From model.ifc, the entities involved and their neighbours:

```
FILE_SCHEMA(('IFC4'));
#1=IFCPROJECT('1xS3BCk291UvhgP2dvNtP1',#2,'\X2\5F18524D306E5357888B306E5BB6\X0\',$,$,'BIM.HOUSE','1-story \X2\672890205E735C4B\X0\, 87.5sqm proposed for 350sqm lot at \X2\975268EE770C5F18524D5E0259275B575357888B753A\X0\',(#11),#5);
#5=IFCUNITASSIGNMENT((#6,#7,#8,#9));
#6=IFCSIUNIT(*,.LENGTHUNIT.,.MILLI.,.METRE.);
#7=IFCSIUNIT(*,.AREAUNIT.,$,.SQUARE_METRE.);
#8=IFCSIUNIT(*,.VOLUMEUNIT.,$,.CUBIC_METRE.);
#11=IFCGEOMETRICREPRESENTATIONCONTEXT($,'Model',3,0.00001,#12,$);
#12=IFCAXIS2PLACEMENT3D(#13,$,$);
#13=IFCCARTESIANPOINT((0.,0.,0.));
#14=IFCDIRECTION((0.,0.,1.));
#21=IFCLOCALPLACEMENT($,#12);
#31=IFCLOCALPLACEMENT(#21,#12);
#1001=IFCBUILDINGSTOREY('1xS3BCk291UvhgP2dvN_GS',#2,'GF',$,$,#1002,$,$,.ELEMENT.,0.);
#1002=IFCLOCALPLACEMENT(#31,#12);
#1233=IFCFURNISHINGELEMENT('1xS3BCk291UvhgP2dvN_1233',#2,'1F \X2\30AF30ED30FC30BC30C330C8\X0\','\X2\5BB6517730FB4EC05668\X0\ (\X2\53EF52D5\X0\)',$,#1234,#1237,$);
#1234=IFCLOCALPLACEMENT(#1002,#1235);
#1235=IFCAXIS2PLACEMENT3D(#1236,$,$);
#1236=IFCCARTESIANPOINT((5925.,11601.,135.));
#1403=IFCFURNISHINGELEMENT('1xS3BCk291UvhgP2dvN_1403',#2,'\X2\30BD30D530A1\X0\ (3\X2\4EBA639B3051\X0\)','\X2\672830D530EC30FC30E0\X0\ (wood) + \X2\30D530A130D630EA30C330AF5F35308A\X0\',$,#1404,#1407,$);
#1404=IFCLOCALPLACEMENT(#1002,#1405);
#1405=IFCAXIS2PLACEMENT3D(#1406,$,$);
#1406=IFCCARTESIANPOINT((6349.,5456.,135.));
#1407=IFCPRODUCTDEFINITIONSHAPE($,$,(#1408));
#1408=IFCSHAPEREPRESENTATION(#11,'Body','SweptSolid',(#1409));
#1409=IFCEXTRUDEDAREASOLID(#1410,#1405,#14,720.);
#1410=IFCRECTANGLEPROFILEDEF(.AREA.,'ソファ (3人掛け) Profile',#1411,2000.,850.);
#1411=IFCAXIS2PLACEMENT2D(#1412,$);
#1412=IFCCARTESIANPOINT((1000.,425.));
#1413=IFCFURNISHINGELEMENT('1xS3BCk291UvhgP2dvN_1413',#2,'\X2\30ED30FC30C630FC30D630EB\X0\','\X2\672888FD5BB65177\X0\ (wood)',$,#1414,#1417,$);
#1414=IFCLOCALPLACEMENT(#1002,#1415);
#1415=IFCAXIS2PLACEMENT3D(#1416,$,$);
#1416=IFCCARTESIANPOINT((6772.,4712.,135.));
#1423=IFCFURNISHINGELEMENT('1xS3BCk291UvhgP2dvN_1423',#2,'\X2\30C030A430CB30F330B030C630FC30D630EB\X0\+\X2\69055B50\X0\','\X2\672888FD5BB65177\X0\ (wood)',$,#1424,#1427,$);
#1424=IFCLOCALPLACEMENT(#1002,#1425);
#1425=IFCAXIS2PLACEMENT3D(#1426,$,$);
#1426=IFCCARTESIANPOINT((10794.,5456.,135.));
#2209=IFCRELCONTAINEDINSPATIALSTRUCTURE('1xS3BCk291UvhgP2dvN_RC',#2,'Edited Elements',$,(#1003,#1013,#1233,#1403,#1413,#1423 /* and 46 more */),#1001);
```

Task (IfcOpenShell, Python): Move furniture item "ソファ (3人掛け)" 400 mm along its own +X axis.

```python
import ifcopenshell
import ifcopenshell.api.geometry
import ifcopenshell.util.placement
import ifcopenshell.util.unit

model = ifcopenshell.open("model.ifc")
unit_scale = ifcopenshell.util.unit.calculate_unit_scale(model)

item = model.by_id(1403)
matrix = ifcopenshell.util.placement.get_local_placement(item.ObjectPlacement)
matrix[:3, 3] += matrix[:3, 0] * 0.4 / unit_scale
ifcopenshell.api.geometry.edit_object_placement(model, product=item, matrix=matrix, is_si=False)

print(ifcopenshell.util.placement.get_local_placement(item.ObjectPlacement).round(3) + 0.0)

model.write("model_rev.ifc")
```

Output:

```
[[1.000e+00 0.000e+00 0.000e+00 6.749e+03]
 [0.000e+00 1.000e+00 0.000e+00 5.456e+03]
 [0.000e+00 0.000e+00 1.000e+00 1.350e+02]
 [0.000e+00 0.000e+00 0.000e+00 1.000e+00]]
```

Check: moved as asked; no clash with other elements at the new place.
